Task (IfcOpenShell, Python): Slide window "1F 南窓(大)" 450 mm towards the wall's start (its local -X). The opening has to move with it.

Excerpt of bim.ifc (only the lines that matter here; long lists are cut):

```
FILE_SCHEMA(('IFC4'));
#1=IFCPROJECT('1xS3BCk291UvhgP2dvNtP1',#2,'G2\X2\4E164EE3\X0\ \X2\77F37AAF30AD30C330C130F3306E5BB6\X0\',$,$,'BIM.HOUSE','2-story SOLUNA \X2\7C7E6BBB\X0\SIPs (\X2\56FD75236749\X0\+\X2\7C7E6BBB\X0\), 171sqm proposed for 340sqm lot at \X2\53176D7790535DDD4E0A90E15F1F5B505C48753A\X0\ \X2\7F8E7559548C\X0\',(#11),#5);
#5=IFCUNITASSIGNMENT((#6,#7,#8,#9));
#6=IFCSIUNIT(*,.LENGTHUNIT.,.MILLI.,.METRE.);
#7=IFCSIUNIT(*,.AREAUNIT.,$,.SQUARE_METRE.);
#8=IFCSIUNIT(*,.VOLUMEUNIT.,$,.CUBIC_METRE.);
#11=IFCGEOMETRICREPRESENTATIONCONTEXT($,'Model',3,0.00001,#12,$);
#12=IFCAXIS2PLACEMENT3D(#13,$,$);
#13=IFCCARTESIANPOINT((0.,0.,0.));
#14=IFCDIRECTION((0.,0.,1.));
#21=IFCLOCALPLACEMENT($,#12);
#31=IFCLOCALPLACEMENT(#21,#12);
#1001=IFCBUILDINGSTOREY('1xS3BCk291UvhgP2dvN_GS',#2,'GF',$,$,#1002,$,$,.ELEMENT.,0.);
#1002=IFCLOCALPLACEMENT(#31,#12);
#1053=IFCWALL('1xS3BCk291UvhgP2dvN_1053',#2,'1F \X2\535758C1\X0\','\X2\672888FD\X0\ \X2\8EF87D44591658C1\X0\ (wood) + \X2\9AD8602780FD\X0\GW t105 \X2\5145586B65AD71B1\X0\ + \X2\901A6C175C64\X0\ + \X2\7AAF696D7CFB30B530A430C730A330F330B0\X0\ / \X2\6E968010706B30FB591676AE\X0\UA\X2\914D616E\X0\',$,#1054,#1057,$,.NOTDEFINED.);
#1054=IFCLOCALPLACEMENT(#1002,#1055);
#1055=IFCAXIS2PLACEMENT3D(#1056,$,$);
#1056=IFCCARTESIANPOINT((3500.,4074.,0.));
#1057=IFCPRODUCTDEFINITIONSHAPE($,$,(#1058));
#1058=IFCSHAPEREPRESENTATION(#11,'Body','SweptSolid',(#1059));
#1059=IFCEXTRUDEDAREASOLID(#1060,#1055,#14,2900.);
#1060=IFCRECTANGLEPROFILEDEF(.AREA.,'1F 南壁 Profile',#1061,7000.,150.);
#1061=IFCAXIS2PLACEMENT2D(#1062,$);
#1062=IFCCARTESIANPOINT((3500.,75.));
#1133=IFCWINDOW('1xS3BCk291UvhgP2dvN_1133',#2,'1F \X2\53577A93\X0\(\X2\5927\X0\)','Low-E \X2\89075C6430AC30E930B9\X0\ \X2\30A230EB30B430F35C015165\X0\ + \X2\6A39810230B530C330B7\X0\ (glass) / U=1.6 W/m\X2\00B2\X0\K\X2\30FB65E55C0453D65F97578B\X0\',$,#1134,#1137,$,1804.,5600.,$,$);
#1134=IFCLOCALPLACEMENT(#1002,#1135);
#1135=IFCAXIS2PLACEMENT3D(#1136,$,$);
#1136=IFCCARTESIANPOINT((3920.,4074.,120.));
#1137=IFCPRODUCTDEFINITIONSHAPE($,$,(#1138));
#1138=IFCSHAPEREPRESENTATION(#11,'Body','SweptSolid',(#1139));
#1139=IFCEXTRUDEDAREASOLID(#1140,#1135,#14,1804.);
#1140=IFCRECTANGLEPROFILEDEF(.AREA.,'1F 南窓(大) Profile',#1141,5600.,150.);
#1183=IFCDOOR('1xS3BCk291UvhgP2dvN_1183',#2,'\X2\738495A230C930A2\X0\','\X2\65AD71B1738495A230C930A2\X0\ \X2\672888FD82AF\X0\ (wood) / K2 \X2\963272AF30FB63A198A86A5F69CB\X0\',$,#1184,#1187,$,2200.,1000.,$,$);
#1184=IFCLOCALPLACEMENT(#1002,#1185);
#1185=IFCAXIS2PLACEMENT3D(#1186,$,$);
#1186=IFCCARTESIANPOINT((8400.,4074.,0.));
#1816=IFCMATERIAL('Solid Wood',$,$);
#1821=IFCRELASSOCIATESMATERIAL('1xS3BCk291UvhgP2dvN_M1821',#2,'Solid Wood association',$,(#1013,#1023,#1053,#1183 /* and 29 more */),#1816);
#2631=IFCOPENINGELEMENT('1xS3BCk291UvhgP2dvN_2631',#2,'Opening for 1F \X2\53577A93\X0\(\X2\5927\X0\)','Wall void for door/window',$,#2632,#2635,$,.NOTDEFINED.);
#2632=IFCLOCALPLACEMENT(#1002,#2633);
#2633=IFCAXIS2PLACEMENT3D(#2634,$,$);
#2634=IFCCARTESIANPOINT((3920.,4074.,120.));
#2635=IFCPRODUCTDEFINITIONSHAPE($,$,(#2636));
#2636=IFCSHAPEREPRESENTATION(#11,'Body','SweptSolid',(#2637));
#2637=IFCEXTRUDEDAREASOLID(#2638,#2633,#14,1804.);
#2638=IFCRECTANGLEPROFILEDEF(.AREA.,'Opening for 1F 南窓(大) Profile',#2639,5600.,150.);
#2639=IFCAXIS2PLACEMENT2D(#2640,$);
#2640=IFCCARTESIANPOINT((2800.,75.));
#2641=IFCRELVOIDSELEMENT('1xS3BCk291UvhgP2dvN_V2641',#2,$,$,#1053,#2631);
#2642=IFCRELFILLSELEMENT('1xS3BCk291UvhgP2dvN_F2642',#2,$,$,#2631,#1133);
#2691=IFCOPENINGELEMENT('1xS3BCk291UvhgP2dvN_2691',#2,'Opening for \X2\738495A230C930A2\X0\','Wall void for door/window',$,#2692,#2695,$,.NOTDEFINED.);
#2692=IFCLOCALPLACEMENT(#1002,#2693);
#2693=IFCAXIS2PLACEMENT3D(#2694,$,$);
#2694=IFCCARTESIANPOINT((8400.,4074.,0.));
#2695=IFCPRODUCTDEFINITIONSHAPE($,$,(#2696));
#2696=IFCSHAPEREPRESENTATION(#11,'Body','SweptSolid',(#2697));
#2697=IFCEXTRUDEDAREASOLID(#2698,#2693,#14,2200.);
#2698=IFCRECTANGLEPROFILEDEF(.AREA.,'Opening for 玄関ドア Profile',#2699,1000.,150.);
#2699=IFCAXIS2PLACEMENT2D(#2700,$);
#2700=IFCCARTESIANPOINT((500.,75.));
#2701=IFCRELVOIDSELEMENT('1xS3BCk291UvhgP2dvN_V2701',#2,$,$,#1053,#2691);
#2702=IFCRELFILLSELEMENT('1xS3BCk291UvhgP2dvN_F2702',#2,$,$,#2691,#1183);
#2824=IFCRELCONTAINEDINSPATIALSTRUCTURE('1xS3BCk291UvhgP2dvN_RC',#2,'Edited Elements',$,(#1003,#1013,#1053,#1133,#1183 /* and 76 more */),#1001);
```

```python
import ifcopenshell
import ifcopenshell.api.geometry
import ifcopenshell.util.placement
import ifcopenshell.util.unit

model = ifcopenshell.open("bim.ifc")
unit_scale = ifcopenshell.util.unit.calculate_unit_scale(model)

window = model.by_guid("1xS3BCk291UvhgP2dvN_1133")
opening = window.FillsVoids[0].RelatingOpeningElement
wall = opening.VoidsElements[0].RelatingBuildingElement

wall_matrix = ifcopenshell.util.placement.get_local_placement(wall.ObjectPlacement)
shift = wall_matrix[:3, 0] * -0.45 / unit_scale
before = ifcopenshell.util.placement.get_local_placement(window.ObjectPlacement)[:3, 3].copy()

# The window is not placed relative to its opening, so move both.
for product in (opening, window):
    matrix = ifcopenshell.util.placement.get_local_placement(product.ObjectPlacement)
    matrix[:3, 3] += shift
    ifcopenshell.api.geometry.edit_object_placement(model, product=product, matrix=matrix, is_si=False)

after = ifcopenshell.util.placement.get_local_placement(window.ObjectPlacement)[:3, 3]
print("window moved by", (after - before).round(3) + 0.0)

model.write("bim_updated.ifc")
```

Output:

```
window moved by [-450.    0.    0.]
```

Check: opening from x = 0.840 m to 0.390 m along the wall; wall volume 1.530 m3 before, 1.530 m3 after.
